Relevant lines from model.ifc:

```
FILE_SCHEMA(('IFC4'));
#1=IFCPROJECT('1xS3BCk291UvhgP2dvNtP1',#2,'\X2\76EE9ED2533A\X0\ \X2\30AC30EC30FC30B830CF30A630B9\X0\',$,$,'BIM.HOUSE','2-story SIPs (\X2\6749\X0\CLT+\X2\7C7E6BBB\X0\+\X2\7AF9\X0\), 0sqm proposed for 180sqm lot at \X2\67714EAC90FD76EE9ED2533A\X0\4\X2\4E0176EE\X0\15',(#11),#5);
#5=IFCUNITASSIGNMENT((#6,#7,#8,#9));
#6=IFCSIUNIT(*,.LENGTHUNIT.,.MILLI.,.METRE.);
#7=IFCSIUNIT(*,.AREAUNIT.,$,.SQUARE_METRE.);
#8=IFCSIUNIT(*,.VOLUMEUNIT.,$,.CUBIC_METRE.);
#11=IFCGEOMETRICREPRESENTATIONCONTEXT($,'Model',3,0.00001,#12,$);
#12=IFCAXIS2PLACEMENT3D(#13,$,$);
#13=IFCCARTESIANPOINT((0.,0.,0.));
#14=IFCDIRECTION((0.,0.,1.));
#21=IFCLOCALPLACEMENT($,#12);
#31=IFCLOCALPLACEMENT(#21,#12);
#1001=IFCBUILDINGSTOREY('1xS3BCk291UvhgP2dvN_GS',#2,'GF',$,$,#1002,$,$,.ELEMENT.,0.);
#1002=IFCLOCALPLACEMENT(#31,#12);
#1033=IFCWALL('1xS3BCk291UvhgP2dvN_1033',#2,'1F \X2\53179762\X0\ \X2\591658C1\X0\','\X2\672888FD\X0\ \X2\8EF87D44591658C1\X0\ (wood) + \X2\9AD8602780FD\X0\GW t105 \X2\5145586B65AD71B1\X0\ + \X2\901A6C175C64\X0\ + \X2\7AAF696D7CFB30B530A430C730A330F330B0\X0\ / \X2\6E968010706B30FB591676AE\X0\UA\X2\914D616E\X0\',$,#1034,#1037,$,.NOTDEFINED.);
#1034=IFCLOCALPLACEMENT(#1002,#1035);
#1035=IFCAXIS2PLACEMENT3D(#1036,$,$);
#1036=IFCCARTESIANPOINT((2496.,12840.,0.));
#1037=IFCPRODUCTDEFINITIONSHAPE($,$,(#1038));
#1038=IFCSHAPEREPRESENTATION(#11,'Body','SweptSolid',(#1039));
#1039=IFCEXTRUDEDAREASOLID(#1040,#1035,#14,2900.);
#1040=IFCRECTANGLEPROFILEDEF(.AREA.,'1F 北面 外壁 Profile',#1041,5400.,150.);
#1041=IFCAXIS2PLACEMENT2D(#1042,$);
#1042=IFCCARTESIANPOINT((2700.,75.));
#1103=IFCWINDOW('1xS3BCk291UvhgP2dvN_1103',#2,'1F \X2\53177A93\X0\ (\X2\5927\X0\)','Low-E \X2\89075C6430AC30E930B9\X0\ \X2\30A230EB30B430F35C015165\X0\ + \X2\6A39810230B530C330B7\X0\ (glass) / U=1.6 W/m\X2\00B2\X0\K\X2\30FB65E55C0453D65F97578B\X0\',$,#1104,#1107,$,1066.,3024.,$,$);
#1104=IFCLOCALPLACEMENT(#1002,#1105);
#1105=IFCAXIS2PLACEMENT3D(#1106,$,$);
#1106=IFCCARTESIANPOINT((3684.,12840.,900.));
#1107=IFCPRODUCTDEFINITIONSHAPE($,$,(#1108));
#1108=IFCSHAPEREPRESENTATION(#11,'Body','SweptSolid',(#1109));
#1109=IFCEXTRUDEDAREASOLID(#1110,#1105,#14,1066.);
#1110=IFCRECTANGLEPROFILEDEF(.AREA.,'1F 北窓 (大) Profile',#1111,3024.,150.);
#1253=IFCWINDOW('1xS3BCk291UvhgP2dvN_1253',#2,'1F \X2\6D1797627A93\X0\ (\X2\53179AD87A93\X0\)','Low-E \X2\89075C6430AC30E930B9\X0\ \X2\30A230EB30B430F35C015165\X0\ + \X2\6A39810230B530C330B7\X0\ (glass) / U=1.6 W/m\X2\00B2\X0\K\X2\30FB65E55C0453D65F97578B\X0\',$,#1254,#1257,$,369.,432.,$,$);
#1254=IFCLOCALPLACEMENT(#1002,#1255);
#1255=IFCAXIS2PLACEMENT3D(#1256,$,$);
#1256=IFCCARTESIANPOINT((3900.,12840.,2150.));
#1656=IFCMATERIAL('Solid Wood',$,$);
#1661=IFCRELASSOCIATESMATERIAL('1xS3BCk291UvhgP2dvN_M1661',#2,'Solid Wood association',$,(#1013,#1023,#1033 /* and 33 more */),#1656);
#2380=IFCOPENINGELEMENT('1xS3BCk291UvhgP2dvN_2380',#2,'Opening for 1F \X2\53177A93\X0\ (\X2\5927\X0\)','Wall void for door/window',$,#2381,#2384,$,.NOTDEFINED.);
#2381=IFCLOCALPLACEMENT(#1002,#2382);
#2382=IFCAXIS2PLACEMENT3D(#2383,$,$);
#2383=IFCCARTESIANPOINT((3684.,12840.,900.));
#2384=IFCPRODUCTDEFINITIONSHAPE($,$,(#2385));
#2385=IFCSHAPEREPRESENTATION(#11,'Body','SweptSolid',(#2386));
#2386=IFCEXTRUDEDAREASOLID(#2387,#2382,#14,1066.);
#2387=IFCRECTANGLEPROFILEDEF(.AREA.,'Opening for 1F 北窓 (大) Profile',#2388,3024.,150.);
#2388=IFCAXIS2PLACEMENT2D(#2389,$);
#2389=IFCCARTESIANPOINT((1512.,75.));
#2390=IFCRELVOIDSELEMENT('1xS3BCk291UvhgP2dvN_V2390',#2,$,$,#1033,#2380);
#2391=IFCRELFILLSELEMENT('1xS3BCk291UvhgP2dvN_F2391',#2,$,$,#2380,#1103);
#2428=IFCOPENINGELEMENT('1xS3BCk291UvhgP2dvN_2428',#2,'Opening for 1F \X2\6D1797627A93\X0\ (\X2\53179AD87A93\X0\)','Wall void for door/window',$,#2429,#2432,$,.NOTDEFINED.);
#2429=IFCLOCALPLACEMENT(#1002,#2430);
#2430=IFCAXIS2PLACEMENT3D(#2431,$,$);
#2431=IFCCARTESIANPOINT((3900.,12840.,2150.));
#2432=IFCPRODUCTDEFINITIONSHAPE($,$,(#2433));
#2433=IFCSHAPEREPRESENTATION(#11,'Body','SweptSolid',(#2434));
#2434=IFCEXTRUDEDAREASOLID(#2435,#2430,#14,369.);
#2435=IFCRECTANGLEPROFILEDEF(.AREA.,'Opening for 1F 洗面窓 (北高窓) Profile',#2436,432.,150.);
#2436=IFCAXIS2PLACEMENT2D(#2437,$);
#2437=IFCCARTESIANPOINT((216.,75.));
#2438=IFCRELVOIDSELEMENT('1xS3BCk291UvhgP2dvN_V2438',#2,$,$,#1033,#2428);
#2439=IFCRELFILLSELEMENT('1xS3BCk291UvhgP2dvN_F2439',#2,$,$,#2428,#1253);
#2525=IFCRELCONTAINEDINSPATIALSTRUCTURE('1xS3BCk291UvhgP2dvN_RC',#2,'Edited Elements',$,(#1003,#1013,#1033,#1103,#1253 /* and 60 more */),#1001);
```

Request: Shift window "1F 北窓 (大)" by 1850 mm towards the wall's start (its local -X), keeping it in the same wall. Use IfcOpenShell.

```python
import ifcopenshell
import ifcopenshell.api.geometry
import ifcopenshell.util.placement
import ifcopenshell.util.unit

model = ifcopenshell.open("model.ifc")
unit_scale = ifcopenshell.util.unit.calculate_unit_scale(model)

window = model.by_id(1103)
opening = window.FillsVoids[0].RelatingOpeningElement
wall = opening.VoidsElements[0].RelatingBuildingElement

wall_matrix = ifcopenshell.util.placement.get_local_placement(wall.ObjectPlacement)
shift = wall_matrix[:3, 0] * -1.85 / unit_scale
before = ifcopenshell.util.placement.get_local_placement(window.ObjectPlacement)[:3, 3].copy()

# The window is not placed relative to its opening, so move both.
for product in (opening, window):
    matrix = ifcopenshell.util.placement.get_local_placement(product.ObjectPlacement)
    matrix[:3, 3] += shift
    ifcopenshell.api.geometry.edit_object_placement(model, product=product, matrix=matrix, is_si=False)

after = ifcopenshell.util.placement.get_local_placement(window.ObjectPlacement)[:3, 3]
print("window moved by", (after - before).round(3) + 0.0)

model.write("model-out.ifc")
```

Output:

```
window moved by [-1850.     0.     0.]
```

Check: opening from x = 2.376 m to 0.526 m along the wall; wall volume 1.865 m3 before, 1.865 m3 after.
